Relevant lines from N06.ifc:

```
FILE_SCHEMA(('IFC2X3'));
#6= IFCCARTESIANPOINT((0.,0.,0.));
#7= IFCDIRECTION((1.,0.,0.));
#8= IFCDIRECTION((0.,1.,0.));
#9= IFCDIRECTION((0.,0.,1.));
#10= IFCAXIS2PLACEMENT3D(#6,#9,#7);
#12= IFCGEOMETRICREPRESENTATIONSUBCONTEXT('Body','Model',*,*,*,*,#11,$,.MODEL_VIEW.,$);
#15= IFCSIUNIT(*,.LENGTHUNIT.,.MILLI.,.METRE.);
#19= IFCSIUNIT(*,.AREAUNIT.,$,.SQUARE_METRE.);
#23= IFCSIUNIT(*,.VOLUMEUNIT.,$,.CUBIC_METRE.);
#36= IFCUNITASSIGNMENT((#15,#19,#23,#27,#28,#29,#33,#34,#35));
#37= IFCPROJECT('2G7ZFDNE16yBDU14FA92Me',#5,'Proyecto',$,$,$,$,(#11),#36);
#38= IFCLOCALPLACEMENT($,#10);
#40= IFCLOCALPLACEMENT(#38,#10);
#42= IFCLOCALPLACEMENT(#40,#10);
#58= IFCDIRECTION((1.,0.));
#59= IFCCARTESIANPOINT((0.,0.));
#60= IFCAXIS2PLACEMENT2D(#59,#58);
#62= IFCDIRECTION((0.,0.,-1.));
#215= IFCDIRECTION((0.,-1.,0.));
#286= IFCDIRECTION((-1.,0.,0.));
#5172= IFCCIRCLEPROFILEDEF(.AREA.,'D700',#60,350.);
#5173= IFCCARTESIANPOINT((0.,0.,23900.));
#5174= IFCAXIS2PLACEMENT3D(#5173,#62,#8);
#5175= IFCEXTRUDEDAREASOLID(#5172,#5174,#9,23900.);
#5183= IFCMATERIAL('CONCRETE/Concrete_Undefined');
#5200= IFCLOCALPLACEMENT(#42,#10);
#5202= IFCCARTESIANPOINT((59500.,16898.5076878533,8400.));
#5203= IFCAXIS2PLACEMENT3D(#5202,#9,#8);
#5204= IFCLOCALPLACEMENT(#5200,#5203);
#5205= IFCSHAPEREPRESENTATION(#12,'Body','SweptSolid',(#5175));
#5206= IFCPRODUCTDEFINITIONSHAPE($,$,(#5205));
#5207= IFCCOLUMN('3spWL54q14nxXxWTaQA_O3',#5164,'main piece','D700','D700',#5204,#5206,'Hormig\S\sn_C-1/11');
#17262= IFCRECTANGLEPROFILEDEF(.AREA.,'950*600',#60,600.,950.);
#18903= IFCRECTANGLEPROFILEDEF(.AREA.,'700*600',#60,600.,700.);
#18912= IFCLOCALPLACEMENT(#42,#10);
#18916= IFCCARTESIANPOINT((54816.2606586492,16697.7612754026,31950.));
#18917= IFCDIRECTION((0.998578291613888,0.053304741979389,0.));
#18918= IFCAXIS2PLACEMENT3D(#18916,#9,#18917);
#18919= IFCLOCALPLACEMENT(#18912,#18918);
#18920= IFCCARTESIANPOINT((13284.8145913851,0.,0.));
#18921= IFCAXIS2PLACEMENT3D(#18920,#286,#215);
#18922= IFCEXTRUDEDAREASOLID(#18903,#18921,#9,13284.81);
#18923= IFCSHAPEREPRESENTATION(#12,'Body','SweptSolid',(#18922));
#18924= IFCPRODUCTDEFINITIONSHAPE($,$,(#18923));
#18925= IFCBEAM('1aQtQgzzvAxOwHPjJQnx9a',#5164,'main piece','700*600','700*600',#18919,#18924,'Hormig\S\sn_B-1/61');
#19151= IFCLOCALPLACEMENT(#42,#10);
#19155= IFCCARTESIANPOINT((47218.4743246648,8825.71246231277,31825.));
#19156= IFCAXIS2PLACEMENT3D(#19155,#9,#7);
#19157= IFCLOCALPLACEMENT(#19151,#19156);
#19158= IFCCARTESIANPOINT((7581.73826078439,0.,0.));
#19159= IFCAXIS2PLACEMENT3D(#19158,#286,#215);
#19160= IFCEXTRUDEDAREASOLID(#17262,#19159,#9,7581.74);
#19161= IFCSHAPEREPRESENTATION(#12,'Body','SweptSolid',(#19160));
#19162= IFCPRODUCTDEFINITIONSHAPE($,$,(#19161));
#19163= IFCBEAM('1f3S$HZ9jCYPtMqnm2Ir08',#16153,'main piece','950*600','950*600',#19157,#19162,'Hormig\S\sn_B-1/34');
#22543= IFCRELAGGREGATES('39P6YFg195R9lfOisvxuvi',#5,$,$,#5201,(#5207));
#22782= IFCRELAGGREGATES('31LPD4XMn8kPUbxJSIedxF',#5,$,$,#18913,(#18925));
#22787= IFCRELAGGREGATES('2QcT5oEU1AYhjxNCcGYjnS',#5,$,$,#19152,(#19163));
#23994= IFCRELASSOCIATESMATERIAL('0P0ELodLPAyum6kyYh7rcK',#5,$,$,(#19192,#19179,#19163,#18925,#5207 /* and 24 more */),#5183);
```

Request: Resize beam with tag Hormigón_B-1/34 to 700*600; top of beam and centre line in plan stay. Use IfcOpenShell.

```python
import ifcopenshell
import ifcopenshell.util.element
import ifcopenshell.util.representation

model = ifcopenshell.open("N06.ifc")

member = model.by_guid("1f3S$HZ9jCYPtMqnm2Ir08")
source = next(p for p in model.by_type("IfcRectangleProfileDef") if p.ProfileName == "700*600")

body = ifcopenshell.util.representation.get_representation(member, "Model", "Body")
solid = body.Items[0]
old_profile = solid.SweptArea

# Copy the section's sizes but keep this member's own profile position.
profile = ifcopenshell.util.element.copy(model, source)
# Profiles are centred, so shift by half the change in depth to hold the top.
shift = (old_profile.YDim - profile.YDim) / 2
x, y = old_profile.Position.Location.Coordinates
up = (0.0, 1.0)  # upwards, in the solid's own plane
location = model.createIfcCartesianPoint((x + up[0] * shift, y + up[1] * shift))
profile.Position = model.createIfcAxis2Placement2D(location, old_profile.Position.RefDirection)
solid.SweptArea = profile
if not model.get_total_inverses(old_profile):
    ifcopenshell.util.element.remove_deep2(model, old_profile)
member.Description = member.Description.replace("950*600", "700*600")
member.ObjectType = member.ObjectType.replace("950*600", "700*600")

print(solid.SweptArea)

model.write("N06_rev.ifc")
```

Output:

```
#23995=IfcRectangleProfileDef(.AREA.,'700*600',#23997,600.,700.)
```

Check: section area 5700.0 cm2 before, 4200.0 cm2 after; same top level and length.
